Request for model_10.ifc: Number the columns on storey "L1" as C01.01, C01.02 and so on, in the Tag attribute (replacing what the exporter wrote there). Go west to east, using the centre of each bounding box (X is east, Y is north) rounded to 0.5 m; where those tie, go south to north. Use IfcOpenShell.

First a look at what the model holds.

```python
import ifcopenshell
import ifcopenshell.util.element
import ifcopenshell.util.placement

model = ifcopenshell.open("model_10.ifc")
print(model.schema)
storey = next(s for s in model.by_type("IfcBuildingStorey") if s.Name == "L1")
columns = [e for e in ifcopenshell.util.element.get_decomposition(storey) if e.is_a("IfcColumn")]
for e in sorted(columns, key=lambda e: e.id()):
    origin = ifcopenshell.util.placement.get_local_placement(e.ObjectPlacement)[:3, 3]
    print(e.id(), e.Tag, e.Name, origin.round(2) + 0.0, sep=" | ")
```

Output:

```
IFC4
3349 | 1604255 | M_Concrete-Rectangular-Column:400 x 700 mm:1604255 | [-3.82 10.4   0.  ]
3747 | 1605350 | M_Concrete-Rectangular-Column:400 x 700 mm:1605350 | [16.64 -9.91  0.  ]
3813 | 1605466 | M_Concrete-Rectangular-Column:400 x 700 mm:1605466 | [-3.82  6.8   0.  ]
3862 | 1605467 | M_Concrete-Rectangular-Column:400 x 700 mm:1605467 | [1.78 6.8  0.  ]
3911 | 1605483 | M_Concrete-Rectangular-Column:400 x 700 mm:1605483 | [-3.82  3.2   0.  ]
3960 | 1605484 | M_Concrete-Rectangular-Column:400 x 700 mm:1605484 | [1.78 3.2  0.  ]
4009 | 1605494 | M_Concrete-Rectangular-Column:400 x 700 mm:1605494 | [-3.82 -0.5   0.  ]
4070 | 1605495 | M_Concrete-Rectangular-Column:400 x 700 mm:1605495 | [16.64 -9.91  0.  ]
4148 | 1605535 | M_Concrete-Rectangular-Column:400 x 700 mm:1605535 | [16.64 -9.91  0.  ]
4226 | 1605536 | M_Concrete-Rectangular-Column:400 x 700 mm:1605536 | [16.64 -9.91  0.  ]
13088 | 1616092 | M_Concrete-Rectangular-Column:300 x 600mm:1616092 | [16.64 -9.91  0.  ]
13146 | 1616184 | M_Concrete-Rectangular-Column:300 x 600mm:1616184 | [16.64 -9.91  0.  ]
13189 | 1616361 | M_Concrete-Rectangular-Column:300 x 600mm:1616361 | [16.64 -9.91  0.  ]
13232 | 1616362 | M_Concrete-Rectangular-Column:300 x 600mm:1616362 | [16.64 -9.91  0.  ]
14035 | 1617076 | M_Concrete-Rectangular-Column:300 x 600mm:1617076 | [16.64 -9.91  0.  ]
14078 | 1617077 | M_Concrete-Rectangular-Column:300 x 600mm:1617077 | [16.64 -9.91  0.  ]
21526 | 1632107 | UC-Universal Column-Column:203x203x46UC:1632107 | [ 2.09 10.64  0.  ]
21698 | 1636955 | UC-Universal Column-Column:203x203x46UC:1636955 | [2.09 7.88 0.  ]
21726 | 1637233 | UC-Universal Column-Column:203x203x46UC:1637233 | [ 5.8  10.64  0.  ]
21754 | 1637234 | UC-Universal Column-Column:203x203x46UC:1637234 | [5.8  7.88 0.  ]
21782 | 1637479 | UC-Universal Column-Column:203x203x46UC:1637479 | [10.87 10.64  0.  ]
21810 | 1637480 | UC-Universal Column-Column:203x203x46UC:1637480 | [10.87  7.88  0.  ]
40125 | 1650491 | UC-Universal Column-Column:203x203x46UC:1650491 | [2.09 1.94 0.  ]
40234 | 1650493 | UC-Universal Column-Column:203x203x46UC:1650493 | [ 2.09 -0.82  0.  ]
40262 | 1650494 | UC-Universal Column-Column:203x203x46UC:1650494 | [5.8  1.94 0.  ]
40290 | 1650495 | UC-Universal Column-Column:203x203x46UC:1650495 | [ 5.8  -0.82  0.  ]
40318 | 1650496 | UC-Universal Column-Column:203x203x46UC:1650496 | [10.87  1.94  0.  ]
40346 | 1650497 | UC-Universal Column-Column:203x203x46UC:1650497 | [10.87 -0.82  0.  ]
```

```python
import ifcopenshell
import ifcopenshell.geom
import ifcopenshell.util.element
import ifcopenshell.util.shape

model = ifcopenshell.open("model_10.ifc")
settings = ifcopenshell.geom.settings()
settings.set("use-world-coords", True)


def centre(element):
    shape = ifcopenshell.geom.create_shape(settings, element)
    return ifcopenshell.util.shape.get_bbox_centroid(shape.geometry)


storey = next(s for s in model.by_type("IfcBuildingStorey") if s.Name == "L1")
columns = [e for e in ifcopenshell.util.element.get_decomposition(storey) if e.is_a("IfcColumn")]

# Insertion points can sit at a corner or the storey origin, so sort by the geometry (in metres).
centres = {e: centre(e) for e in columns}
columns.sort(key=lambda e: (round(centres[e][0] / 0.5), centres[e][1]))

for i, e in enumerate(columns, start=1):
    number = f"C01.{i:02d}"
    e.Tag = number
    print(e.id(), number)

model.write("model_10_v2.ifc")
```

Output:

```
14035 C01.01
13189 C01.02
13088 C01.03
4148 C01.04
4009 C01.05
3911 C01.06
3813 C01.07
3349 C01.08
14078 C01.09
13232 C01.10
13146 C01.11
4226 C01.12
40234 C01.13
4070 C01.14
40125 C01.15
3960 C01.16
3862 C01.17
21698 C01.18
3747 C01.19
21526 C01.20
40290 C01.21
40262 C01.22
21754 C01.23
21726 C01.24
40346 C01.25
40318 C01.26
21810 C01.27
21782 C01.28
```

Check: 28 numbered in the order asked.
